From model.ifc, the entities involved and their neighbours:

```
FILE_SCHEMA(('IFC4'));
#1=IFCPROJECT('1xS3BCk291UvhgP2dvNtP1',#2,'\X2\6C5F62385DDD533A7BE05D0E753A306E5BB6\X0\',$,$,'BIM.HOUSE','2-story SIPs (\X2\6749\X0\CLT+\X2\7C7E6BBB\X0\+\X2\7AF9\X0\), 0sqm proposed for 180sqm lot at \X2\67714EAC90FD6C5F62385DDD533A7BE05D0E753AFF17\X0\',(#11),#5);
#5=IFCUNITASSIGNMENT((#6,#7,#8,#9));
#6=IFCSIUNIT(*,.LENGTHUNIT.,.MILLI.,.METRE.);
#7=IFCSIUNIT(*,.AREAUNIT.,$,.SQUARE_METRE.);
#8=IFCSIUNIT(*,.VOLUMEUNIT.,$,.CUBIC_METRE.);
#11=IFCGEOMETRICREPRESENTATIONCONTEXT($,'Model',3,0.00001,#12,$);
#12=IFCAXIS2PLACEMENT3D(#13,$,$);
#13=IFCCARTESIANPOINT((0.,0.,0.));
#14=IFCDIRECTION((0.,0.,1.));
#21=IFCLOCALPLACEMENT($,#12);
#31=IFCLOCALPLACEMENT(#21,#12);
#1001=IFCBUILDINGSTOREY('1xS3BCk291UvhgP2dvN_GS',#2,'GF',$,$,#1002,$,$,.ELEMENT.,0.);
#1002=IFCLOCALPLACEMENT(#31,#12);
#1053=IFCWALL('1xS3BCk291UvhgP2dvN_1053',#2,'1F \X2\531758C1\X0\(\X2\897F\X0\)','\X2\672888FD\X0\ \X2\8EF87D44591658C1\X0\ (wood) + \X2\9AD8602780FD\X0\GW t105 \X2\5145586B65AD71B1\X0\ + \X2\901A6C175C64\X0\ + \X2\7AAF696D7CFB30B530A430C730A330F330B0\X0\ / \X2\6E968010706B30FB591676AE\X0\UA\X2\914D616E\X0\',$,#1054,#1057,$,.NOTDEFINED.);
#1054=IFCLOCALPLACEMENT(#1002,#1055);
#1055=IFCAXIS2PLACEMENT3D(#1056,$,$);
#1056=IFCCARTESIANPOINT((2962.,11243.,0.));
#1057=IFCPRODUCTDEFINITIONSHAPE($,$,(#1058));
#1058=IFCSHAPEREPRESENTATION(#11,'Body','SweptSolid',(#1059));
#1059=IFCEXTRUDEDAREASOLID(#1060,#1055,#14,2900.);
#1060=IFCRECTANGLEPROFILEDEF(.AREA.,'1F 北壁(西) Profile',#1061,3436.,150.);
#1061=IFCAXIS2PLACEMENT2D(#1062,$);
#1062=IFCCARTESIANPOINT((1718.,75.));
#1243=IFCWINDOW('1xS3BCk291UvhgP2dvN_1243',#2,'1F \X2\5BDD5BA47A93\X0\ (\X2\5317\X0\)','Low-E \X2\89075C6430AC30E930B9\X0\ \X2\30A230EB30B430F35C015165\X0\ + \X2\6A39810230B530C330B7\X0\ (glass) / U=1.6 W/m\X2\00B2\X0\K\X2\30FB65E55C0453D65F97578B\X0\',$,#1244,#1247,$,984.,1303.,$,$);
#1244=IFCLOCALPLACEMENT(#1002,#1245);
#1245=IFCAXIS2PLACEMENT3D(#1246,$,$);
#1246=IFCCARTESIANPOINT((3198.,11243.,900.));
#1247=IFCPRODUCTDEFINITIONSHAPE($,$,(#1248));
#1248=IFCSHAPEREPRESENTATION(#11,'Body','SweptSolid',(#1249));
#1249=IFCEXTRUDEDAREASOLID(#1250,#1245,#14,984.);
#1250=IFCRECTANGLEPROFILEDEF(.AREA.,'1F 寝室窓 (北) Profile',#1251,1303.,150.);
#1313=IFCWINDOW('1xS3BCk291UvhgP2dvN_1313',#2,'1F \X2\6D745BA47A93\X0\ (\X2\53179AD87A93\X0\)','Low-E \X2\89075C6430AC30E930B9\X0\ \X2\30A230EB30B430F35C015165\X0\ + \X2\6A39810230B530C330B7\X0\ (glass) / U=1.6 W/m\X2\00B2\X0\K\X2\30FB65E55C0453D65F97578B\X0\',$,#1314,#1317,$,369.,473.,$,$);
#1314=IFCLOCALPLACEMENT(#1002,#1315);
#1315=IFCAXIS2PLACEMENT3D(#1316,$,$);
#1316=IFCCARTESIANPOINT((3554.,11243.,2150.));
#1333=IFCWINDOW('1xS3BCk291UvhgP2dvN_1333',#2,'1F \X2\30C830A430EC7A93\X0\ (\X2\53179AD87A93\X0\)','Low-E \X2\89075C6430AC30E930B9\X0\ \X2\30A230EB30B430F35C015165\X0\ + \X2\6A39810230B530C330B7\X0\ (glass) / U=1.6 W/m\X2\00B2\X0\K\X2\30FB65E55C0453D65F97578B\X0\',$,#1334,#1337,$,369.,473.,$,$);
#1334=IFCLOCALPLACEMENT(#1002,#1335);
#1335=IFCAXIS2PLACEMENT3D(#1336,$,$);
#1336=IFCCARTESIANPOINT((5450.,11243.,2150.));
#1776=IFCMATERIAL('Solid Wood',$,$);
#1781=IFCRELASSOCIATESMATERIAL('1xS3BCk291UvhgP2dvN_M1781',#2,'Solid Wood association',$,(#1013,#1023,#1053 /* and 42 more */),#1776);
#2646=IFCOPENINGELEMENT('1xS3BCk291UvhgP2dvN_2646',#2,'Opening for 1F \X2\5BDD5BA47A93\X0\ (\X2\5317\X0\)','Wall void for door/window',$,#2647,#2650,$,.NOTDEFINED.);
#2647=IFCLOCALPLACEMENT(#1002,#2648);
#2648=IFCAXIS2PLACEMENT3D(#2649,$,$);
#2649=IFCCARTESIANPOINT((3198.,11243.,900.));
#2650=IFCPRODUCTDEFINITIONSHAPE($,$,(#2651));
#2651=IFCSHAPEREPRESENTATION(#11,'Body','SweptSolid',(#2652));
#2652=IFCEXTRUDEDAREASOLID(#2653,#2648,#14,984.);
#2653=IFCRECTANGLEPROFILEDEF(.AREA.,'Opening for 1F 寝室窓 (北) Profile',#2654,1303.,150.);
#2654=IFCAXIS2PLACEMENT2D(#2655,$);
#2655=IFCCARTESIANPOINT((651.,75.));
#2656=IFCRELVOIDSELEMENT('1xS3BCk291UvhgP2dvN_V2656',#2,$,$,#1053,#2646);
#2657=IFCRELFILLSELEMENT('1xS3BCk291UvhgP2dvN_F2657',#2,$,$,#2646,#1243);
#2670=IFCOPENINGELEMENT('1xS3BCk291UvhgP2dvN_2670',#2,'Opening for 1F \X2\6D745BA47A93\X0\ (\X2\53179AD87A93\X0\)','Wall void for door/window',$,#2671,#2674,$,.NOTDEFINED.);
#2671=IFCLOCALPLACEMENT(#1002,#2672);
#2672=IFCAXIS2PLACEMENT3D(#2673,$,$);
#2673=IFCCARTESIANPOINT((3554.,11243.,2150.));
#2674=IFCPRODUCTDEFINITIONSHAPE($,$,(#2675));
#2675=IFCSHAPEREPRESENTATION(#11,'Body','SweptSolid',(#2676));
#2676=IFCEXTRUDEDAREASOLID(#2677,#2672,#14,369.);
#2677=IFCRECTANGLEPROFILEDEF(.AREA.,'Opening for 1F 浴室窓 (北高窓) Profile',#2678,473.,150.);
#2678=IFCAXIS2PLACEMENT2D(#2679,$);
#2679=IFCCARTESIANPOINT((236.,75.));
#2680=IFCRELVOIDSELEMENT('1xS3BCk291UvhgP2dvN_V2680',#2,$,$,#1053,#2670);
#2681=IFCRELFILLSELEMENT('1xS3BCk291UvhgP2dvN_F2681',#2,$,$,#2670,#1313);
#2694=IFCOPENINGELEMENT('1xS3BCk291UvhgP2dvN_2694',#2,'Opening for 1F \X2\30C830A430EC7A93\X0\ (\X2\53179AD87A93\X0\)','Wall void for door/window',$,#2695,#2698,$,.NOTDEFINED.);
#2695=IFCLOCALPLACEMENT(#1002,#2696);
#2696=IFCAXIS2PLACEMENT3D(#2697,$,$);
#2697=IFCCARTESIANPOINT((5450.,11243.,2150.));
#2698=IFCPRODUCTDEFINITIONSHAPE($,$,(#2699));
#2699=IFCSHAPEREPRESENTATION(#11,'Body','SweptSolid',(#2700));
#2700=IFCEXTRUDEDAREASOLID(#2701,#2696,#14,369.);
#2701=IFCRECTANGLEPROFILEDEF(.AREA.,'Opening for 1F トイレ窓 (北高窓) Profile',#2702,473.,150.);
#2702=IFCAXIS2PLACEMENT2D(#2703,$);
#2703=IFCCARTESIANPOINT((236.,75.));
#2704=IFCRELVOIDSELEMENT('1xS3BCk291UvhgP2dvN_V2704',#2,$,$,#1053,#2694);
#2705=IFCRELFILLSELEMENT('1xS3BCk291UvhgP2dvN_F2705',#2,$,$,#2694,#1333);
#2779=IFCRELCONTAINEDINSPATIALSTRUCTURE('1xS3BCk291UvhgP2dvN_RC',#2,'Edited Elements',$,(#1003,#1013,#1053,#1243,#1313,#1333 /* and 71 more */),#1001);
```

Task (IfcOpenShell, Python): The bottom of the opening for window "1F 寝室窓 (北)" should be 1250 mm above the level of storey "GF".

```python
import numpy as np
import ifcopenshell
import ifcopenshell.api.geometry
import ifcopenshell.geom
import ifcopenshell.util.element
import ifcopenshell.util.placement
import ifcopenshell.util.shape
import ifcopenshell.util.unit

model = ifcopenshell.open("model.ifc")
unit_scale = ifcopenshell.util.unit.calculate_unit_scale(model)

window = model.by_guid("1xS3BCk291UvhgP2dvN_1243")
opening = window.FillsVoids[0].RelatingOpeningElement
storey = ifcopenshell.util.element.get_container(window, ifc_class="IfcBuildingStorey")
level = ifcopenshell.util.placement.get_local_placement(storey.ObjectPlacement)[2, 3]

# The opening's origin need not be at the sill, so measure its lowest point.
shape = ifcopenshell.geom.create_shape(ifcopenshell.geom.settings(), opening)
bottom = ifcopenshell.util.shape.get_shape_bottom_elevation(shape, shape.geometry) / unit_scale
dz = level + 1.25 / unit_scale - bottom

shift = np.array([0.0, 0.0, dz])
# The window is not placed relative to its opening, so move both.
for product in (opening, window):
    matrix = ifcopenshell.util.placement.get_local_placement(product.ObjectPlacement)
    matrix[:3, 3] += shift
    ifcopenshell.api.geometry.edit_object_placement(model, product=product, matrix=matrix, is_si=False)

print(f"moved by {dz * unit_scale:+.3f} m")

model.write("model_edited.ifc")
```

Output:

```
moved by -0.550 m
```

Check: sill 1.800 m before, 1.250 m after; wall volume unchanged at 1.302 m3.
